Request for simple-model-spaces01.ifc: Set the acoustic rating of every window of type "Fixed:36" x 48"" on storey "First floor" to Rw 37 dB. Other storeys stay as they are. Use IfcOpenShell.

First a look at what the model holds.

```python
import ifcopenshell
import ifcopenshell.util.element

model = ifcopenshell.open("simple-model-spaces01.ifc")
print(model.schema)
storey = next(s for s in model.by_type("IfcBuildingStorey") if s.Name == "First floor")
windows = [e for e in ifcopenshell.util.element.get_decomposition(storey) if e.is_a("IfcWindow")]
seen = {}
for e in windows:
    element_type = ifcopenshell.util.element.get_type(e)
    key = (element_type.Name if element_type != e and element_type else None, ifcopenshell.util.element.get_pset(e, "Pset_WindowCommon", "AcousticRating"))
    seen[key] = seen.get(key, 0) + 1
for (name, value), count in sorted(seen.items(), key=str):
    print(count, "x", name, "|", value)
```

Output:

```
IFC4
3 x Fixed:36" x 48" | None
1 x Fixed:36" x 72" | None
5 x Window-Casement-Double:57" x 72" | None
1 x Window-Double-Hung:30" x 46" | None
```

```python
import ifcopenshell
import ifcopenshell.api.pset
import ifcopenshell.util.element

model = ifcopenshell.open("simple-model-spaces01.ifc")

storey = next(s for s in model.by_type("IfcBuildingStorey") if s.Name == "First floor")
windows = [e for e in ifcopenshell.util.element.get_decomposition(storey) if e.is_a("IfcWindow")]

count = 0
for e in windows:
    element_type = ifcopenshell.util.element.get_type(e)
    if element_type in (None, e) or element_type.Name != 'Fixed:36" x 48"':
        continue
    # add_pset returns the element's existing set when there is one.
    pset = ifcopenshell.api.pset.add_pset(model, product=e, name="Pset_WindowCommon")
    ifcopenshell.api.pset.edit_pset(model, pset=pset, properties={"AcousticRating": "Rw 37 dB"})
    count += 1

print(count, "windows updated")

model.write("simple-model-spaces01-out.ifc")
```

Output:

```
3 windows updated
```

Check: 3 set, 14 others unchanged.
